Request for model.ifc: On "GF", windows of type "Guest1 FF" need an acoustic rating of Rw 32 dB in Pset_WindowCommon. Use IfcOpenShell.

First a look at what the model holds.

```python
import ifcopenshell
import ifcopenshell.util.element

model = ifcopenshell.open("model.ifc")
print(model.schema)
storey = next(s for s in model.by_type("IfcBuildingStorey") if s.Name == "GF")
windows = [e for e in ifcopenshell.util.element.get_decomposition(storey) if e.is_a("IfcWindow")]
seen = {}
for e in windows:
    element_type = ifcopenshell.util.element.get_type(e)
    key = (element_type.Name if element_type != e and element_type else None, ifcopenshell.util.element.get_pset(e, "Pset_WindowCommon", "AcousticRating"))
    seen[key] = seen.get(key, 0) + 1
for (name, value), count in sorted(seen.items(), key=str):
    print(count, "x", name, "|", value)
```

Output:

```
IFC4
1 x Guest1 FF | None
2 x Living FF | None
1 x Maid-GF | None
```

```python
import ifcopenshell
import ifcopenshell.api.pset
import ifcopenshell.util.element

model = ifcopenshell.open("model.ifc")

storey = next(s for s in model.by_type("IfcBuildingStorey") if s.Name == "GF")
windows = [e for e in ifcopenshell.util.element.get_decomposition(storey) if e.is_a("IfcWindow")]

count = 0
for e in windows:
    element_type = ifcopenshell.util.element.get_type(e)
    if element_type in (None, e) or element_type.Name != "Guest1 FF":
        continue
    # add_pset returns the element's existing set when there is one.
    pset = ifcopenshell.api.pset.add_pset(model, product=e, name="Pset_WindowCommon")
    ifcopenshell.api.pset.edit_pset(model, pset=pset, properties={"AcousticRating": "Rw 32 dB"})
    count += 1

print(count, "windows updated")

model.write("model_v2.ifc")
```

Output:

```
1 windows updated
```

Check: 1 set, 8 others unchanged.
